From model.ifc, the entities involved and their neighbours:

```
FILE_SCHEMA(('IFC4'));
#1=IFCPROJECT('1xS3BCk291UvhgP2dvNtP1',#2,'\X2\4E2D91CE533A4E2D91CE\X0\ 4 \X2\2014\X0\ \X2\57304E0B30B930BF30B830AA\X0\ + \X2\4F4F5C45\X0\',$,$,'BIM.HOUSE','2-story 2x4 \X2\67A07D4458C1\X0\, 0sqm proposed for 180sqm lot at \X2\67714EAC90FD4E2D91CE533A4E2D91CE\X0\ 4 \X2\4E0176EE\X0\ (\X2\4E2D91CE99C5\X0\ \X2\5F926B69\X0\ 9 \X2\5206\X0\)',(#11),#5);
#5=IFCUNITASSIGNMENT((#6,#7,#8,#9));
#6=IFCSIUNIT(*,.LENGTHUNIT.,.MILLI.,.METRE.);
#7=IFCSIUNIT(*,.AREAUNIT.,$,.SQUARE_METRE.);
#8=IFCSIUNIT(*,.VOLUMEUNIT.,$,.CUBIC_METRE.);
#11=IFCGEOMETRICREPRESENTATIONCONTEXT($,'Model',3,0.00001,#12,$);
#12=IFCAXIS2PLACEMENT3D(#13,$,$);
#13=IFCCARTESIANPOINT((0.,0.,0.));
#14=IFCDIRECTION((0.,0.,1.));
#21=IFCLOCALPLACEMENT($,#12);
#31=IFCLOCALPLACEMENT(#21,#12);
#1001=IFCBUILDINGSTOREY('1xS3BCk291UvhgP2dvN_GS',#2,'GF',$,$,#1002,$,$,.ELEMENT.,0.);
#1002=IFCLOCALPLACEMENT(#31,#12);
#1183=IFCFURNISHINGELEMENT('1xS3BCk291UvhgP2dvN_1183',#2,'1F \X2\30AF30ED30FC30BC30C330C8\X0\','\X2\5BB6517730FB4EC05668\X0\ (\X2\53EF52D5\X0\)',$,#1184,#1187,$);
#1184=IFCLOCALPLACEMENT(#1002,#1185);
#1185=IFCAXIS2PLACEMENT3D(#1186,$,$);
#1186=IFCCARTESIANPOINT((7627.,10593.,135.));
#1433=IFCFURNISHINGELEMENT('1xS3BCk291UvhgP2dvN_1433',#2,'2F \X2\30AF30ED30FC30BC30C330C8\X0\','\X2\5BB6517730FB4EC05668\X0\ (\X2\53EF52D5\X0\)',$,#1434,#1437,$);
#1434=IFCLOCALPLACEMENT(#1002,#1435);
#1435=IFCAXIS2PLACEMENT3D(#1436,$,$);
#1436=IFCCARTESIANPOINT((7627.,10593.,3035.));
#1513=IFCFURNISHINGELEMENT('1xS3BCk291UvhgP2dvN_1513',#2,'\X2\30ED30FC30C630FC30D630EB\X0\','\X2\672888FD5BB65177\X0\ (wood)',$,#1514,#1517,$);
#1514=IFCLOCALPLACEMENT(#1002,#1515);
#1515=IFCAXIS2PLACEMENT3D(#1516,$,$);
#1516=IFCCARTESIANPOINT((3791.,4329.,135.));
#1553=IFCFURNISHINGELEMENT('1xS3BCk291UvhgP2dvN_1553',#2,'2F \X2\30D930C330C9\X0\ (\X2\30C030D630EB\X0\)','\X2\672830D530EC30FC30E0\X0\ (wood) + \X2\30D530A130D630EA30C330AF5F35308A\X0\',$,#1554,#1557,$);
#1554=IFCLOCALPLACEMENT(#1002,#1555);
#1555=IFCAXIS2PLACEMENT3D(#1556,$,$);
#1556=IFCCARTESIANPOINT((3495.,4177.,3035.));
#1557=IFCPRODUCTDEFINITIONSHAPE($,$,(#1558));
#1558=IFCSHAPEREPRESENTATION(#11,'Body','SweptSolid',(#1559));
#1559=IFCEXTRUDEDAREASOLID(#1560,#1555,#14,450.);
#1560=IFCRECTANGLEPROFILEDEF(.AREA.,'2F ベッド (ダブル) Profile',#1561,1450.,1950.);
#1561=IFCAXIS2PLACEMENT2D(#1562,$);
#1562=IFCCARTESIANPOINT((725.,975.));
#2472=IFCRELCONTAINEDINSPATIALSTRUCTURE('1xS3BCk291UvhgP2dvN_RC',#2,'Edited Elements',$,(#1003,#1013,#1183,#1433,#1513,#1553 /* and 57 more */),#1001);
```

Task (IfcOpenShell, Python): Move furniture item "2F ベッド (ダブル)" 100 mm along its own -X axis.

```python
import ifcopenshell
import ifcopenshell.api.geometry
import ifcopenshell.util.placement

model = ifcopenshell.open("model.ifc")

item = model.by_guid("1xS3BCk291UvhgP2dvN_1553")
matrix = ifcopenshell.util.placement.get_local_placement(item.ObjectPlacement)
matrix[:3, 3] -= matrix[:3, 0] * 100.0
ifcopenshell.api.geometry.edit_object_placement(model, product=item, matrix=matrix, is_si=False)

print(ifcopenshell.util.placement.get_local_placement(item.ObjectPlacement).round(3) + 0.0)

model.write("model_edited.ifc")
```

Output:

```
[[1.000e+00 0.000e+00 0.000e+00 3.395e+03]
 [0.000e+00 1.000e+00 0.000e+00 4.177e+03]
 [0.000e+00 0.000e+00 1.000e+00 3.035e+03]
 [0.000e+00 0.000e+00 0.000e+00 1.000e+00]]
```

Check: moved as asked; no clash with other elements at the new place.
